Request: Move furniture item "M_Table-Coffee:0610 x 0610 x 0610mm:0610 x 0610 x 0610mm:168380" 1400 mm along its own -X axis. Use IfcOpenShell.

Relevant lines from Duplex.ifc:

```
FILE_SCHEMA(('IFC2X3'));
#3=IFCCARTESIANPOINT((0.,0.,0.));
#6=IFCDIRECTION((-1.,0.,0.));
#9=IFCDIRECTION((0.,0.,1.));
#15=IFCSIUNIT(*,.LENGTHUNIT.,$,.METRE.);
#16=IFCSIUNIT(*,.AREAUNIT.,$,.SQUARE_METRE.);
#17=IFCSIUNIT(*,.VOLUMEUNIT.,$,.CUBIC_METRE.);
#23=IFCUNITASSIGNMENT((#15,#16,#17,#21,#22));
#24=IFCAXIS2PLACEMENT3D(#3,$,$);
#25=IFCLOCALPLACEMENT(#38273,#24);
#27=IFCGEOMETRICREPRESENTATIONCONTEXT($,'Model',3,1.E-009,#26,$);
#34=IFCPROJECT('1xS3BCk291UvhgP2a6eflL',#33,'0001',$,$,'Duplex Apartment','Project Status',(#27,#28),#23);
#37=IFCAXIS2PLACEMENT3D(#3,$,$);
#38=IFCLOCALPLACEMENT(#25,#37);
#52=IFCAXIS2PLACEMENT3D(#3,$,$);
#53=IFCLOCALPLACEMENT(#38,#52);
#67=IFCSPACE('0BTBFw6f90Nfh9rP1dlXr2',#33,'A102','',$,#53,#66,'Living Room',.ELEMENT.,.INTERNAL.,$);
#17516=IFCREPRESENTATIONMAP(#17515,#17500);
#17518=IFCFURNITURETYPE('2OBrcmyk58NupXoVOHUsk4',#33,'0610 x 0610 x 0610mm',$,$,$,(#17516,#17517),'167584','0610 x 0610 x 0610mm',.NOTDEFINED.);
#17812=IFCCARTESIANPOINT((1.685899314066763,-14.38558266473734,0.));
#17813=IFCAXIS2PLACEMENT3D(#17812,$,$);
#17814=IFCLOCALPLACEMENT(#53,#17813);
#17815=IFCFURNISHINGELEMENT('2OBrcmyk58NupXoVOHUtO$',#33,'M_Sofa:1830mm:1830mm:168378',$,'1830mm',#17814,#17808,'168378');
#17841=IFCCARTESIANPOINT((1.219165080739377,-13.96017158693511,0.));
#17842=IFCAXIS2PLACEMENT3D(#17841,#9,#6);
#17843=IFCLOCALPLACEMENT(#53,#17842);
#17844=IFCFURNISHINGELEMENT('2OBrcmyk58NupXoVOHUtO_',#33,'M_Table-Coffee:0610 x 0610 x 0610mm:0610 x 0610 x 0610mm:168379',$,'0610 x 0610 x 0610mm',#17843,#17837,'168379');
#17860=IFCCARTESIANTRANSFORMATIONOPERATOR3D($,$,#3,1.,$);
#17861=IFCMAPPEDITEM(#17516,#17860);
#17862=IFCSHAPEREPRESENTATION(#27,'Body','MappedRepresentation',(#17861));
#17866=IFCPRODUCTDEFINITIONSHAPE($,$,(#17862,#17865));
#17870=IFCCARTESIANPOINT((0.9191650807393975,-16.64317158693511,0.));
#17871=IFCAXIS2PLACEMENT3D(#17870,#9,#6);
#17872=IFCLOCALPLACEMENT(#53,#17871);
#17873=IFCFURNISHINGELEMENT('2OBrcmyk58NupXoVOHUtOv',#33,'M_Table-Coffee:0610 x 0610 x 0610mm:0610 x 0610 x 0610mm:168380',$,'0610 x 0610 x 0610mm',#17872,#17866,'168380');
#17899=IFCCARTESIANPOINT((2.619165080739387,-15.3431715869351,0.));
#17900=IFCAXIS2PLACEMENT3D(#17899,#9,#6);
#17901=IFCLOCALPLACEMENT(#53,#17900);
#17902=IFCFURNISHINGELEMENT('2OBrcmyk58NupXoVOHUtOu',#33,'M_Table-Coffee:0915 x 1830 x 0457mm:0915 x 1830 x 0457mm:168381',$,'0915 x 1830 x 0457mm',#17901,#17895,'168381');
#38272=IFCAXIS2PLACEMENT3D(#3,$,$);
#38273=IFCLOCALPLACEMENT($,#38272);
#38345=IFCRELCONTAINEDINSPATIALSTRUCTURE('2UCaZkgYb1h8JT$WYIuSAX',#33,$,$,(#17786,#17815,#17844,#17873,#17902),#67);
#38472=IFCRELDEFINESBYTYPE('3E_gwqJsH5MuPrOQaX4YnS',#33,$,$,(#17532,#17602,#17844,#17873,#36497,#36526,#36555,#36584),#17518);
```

```python
import ifcopenshell
import ifcopenshell.api.geometry
import ifcopenshell.util.placement
import ifcopenshell.util.unit

model = ifcopenshell.open("Duplex.ifc")
unit_scale = ifcopenshell.util.unit.calculate_unit_scale(model)

item = model.by_guid("2OBrcmyk58NupXoVOHUtOv")
matrix = ifcopenshell.util.placement.get_local_placement(item.ObjectPlacement)
matrix[:3, 3] -= matrix[:3, 0] * 1.4 / unit_scale
ifcopenshell.api.geometry.edit_object_placement(model, product=item, matrix=matrix, is_si=False)

print(ifcopenshell.util.placement.get_local_placement(item.ObjectPlacement).round(3) + 0.0)

model.write("Duplex_v2.ifc")
```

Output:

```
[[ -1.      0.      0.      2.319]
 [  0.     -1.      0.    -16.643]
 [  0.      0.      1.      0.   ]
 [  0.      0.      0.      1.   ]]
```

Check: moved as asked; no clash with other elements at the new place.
